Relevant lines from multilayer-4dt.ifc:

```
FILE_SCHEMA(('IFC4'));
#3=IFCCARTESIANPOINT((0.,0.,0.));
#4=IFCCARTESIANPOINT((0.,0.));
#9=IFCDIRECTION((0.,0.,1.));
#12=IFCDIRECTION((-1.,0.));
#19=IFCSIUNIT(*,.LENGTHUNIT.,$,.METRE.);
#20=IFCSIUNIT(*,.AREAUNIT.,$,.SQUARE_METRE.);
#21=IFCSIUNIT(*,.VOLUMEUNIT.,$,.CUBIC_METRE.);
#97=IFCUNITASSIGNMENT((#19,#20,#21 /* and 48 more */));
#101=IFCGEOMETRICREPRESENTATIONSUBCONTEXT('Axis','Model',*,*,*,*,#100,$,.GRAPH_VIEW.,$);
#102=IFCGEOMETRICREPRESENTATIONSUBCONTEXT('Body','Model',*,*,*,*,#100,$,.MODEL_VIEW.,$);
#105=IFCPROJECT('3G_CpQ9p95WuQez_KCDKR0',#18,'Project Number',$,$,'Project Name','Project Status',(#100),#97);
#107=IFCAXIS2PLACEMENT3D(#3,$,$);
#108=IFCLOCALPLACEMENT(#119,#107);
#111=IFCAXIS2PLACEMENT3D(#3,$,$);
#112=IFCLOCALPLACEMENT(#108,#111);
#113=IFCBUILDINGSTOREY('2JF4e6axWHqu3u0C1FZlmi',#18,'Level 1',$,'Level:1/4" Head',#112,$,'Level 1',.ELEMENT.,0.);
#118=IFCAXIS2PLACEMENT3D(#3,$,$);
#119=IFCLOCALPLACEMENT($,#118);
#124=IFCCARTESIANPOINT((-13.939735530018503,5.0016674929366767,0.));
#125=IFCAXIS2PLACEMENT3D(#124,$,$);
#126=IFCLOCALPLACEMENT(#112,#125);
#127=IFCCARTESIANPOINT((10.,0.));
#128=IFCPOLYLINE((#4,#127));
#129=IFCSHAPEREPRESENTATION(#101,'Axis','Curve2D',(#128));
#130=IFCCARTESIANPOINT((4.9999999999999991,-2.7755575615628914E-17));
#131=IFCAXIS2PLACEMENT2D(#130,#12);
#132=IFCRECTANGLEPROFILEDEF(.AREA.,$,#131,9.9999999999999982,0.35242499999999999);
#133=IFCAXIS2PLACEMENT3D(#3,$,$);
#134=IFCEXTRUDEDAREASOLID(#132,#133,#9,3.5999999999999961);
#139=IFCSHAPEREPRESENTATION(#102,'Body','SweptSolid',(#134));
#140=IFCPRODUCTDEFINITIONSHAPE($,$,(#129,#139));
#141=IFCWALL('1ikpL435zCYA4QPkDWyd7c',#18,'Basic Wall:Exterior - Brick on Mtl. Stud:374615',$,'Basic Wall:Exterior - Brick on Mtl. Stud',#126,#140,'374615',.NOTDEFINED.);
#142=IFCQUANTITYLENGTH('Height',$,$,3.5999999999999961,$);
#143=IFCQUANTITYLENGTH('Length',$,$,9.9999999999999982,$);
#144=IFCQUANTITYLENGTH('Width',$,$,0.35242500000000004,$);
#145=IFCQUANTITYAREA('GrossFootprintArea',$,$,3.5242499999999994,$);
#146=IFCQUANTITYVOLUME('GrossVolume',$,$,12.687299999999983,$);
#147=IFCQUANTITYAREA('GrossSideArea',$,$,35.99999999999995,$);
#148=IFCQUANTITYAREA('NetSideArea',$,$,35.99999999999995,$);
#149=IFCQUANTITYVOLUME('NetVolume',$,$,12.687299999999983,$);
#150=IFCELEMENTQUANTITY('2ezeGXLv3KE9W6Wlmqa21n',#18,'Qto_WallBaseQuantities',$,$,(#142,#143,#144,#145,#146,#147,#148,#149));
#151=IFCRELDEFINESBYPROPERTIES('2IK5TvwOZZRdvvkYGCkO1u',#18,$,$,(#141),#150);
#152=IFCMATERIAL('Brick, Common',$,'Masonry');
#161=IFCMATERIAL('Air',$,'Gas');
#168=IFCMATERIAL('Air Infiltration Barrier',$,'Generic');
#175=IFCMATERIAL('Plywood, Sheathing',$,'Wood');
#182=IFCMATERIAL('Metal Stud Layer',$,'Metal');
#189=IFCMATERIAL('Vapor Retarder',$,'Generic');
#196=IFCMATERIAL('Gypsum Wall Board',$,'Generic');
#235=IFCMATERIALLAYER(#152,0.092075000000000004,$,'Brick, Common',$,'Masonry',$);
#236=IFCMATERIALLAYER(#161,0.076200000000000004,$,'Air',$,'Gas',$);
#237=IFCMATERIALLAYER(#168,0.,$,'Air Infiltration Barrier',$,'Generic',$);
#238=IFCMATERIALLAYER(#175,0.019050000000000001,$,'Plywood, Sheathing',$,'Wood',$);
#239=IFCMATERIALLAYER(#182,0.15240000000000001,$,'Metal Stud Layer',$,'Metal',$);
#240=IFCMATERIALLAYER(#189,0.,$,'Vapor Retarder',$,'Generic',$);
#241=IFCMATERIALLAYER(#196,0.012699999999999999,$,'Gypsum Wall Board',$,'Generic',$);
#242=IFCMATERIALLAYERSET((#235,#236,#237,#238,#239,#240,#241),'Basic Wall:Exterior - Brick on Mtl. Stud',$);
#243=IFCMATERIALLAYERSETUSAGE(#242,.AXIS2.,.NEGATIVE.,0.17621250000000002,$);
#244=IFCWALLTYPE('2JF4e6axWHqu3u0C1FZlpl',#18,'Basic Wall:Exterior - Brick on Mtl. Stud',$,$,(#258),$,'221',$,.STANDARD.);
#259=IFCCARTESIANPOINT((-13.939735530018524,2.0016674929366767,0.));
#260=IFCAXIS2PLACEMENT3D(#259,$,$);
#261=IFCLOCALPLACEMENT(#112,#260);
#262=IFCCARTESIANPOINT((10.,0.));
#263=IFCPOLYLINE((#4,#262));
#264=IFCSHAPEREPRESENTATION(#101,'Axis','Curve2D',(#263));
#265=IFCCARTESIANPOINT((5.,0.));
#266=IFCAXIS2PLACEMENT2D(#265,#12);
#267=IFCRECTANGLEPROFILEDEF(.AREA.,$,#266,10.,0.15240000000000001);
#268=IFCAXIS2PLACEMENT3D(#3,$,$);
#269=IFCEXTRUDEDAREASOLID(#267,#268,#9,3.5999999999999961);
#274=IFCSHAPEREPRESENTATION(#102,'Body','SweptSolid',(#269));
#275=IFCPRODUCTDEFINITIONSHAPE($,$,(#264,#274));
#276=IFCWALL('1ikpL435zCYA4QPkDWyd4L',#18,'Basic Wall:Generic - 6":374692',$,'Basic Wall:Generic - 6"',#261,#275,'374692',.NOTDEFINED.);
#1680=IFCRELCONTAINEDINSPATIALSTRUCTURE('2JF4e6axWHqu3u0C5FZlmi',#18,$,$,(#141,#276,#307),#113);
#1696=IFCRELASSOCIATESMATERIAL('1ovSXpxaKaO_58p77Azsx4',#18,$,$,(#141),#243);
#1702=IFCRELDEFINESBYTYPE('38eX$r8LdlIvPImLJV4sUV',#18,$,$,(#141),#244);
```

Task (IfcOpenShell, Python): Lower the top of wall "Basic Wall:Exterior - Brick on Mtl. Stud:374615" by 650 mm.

```python
import ifcopenshell
import ifcopenshell.api.pset
import ifcopenshell.geom
import ifcopenshell.util.element
import ifcopenshell.util.representation
import ifcopenshell.util.shape
import ifcopenshell.util.unit

model = ifcopenshell.open("multilayer-4dt.ifc")
unit_scale = ifcopenshell.util.unit.calculate_unit_scale(model)
area_scale = ifcopenshell.util.unit.calculate_unit_scale(model, "AREAUNIT")
volume_scale = ifcopenshell.util.unit.calculate_unit_scale(model, "VOLUMEUNIT")
settings = ifcopenshell.geom.settings()


def volume(element):
    """Net volume in cubic metres, openings subtracted."""
    shape = ifcopenshell.geom.create_shape(settings, element)
    return ifcopenshell.util.shape.get_volume(shape.geometry)


wall = model.by_id(141)
before = volume(wall)

body = ifcopenshell.util.representation.get_representation(wall, "Model", "Body")
solid = body.Items[0]
old_height = solid.Depth
solid.Depth -= 0.65 / unit_scale
after = volume(wall)
thickness = 0.3524  # wall thickness in metres

# Update the stored height, areas and volumes.
qto = model.by_id(ifcopenshell.util.element.get_pset(wall, "Qto_WallBaseQuantities", should_inherit=False)["id"])
ifcopenshell.api.pset.edit_qto(model, qto=qto, properties={
    "Height": solid.Depth,
    "GrossVolume": ifcopenshell.util.element.get_pset(wall, "Qto_WallBaseQuantities", "GrossVolume") * solid.Depth / old_height,
    "GrossSideArea": ifcopenshell.util.element.get_pset(wall, "Qto_WallBaseQuantities", "GrossSideArea") * solid.Depth / old_height,
    "NetSideArea": after / thickness / area_scale,
    "NetVolume": after / volume_scale,
})

print(f"height {old_height:g} -> {solid.Depth:g}, volume {before:.3f} -> {after:.3f} m3")

model.write("multilayer-4dt_rev.ifc")
```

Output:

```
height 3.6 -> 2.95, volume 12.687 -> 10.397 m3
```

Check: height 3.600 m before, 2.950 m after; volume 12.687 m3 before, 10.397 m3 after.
